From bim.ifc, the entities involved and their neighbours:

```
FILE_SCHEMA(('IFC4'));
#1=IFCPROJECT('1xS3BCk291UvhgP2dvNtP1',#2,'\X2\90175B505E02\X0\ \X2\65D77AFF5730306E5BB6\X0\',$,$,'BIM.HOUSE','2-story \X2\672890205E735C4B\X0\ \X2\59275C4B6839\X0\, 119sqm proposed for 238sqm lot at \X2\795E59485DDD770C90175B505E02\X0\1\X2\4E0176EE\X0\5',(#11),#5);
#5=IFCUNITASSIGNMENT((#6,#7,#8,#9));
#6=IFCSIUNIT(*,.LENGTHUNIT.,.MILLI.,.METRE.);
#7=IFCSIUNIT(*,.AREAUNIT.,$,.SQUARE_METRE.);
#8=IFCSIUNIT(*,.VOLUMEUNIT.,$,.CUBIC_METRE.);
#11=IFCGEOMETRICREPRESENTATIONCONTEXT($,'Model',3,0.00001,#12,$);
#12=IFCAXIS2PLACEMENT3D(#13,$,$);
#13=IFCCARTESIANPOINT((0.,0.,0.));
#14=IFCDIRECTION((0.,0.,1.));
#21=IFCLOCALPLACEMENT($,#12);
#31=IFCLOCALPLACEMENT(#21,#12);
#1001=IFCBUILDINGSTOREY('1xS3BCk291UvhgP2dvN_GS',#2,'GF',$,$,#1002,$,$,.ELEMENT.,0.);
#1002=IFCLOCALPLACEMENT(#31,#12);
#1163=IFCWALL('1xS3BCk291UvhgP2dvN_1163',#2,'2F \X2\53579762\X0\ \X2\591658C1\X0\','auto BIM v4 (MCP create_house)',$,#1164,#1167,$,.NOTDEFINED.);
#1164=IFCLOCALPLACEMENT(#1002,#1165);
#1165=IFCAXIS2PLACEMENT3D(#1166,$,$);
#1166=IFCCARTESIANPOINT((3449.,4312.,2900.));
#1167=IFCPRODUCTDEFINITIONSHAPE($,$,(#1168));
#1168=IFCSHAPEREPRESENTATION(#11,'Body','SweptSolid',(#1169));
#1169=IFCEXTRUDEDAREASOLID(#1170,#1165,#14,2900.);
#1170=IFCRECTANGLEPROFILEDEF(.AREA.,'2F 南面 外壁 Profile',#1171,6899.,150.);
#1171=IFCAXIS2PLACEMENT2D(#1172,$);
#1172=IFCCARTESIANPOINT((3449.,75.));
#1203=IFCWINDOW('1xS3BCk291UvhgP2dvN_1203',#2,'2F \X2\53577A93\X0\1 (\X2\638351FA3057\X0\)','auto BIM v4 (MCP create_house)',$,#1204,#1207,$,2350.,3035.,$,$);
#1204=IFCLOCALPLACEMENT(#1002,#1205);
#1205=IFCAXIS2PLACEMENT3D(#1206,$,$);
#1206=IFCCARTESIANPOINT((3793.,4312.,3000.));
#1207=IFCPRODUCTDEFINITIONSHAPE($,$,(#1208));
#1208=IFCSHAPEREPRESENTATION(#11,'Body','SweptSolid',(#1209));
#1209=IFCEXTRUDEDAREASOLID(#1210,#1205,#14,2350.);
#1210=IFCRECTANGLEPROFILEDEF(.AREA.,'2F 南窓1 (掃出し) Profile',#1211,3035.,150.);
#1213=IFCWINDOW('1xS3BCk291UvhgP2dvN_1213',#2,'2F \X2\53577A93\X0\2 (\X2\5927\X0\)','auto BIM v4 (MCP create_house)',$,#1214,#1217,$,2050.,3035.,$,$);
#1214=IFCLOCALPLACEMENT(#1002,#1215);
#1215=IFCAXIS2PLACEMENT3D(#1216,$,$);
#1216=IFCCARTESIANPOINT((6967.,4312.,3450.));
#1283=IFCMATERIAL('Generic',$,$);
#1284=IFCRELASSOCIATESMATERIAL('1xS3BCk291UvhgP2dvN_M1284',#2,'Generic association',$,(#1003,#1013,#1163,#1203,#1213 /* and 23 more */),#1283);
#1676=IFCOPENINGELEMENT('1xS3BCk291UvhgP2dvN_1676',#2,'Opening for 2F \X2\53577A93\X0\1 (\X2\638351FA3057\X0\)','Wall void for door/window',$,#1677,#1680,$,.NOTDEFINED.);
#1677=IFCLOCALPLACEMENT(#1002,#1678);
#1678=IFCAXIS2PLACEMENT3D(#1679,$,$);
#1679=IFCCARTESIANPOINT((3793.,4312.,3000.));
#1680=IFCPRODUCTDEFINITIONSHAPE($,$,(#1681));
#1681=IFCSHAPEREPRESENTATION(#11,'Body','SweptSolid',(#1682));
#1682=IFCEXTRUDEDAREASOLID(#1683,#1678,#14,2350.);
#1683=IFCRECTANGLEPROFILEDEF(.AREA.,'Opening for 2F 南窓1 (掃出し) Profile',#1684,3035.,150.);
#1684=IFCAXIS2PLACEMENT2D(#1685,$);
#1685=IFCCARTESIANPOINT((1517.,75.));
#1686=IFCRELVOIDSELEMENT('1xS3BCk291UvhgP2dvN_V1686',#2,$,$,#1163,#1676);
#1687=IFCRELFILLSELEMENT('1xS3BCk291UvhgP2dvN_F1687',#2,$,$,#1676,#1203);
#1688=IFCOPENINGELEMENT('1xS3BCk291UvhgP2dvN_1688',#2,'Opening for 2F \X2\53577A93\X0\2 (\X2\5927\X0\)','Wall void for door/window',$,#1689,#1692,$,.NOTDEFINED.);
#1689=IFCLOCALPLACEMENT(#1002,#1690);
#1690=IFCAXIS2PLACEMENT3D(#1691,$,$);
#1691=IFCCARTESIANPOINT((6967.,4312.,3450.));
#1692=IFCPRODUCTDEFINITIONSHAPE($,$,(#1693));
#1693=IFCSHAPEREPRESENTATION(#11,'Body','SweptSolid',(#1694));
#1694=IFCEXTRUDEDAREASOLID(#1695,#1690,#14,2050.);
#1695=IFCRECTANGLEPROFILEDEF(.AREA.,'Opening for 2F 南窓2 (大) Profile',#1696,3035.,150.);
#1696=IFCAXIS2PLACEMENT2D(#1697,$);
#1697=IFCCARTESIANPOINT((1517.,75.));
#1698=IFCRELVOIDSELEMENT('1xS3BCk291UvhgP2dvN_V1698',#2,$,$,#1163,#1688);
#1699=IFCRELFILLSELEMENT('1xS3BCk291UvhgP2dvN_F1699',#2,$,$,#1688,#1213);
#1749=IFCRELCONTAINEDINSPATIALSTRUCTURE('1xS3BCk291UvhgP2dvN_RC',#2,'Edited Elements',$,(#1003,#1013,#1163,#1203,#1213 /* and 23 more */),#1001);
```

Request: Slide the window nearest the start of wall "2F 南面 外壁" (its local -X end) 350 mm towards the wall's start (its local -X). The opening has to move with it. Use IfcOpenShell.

```python
import ifcopenshell
import ifcopenshell.api.geometry
import ifcopenshell.util.placement

model = ifcopenshell.open("bim.ifc")

window = model.by_guid("1xS3BCk291UvhgP2dvN_1203")
opening = window.FillsVoids[0].RelatingOpeningElement
wall = opening.VoidsElements[0].RelatingBuildingElement

wall_matrix = ifcopenshell.util.placement.get_local_placement(wall.ObjectPlacement)
shift = wall_matrix[:3, 0] * -350.0
before = ifcopenshell.util.placement.get_local_placement(window.ObjectPlacement)[:3, 3].copy()

# The window is not placed relative to its opening, so move both.
for product in (opening, window):
    matrix = ifcopenshell.util.placement.get_local_placement(product.ObjectPlacement)
    matrix[:3, 3] += shift
    ifcopenshell.api.geometry.edit_object_placement(model, product=product, matrix=matrix, is_si=False)

after = ifcopenshell.util.placement.get_local_placement(window.ObjectPlacement)[:3, 3]
print("window moved by", (after - before).round(3) + 0.0)

model.write("bim_rev.ifc")
```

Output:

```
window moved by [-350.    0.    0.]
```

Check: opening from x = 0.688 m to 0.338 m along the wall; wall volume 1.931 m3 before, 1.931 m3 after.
